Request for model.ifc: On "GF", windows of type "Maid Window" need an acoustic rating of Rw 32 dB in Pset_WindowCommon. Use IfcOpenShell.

First a look at what the model holds.

```python
import ifcopenshell
import ifcopenshell.util.element

model = ifcopenshell.open("model.ifc")
print(model.schema)
storey = next(s for s in model.by_type("IfcBuildingStorey") if s.Name == "GF")
windows = [e for e in ifcopenshell.util.element.get_decomposition(storey) if e.is_a("IfcWindow")]
seen = {}
for e in windows:
    element_type = ifcopenshell.util.element.get_type(e)
    key = (element_type.Name if element_type != e and element_type else None, ifcopenshell.util.element.get_pset(e, "Pset_WindowCommon", "AcousticRating"))
    seen[key] = seen.get(key, 0) + 1
for (name, value), count in sorted(seen.items(), key=str):
    print(count, "x", name, "|", value)
```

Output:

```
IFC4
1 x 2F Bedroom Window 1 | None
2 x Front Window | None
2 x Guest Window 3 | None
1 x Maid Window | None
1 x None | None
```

```python
import ifcopenshell
import ifcopenshell.api.pset
import ifcopenshell.util.element

model = ifcopenshell.open("model.ifc")

storey = next(s for s in model.by_type("IfcBuildingStorey") if s.Name == "GF")
windows = [e for e in ifcopenshell.util.element.get_decomposition(storey) if e.is_a("IfcWindow")]

count = 0
for e in windows:
    element_type = ifcopenshell.util.element.get_type(e)
    if element_type in (None, e) or element_type.Name != "Maid Window":
        continue
    # add_pset returns the element's existing set when there is one.
    pset = ifcopenshell.api.pset.add_pset(model, product=e, name="Pset_WindowCommon")
    ifcopenshell.api.pset.edit_pset(model, pset=pset, properties={"AcousticRating": "Rw 32 dB"})
    count += 1

print(count, "windows updated")

model.write("model_updated.ifc")
```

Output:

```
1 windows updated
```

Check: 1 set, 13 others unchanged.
